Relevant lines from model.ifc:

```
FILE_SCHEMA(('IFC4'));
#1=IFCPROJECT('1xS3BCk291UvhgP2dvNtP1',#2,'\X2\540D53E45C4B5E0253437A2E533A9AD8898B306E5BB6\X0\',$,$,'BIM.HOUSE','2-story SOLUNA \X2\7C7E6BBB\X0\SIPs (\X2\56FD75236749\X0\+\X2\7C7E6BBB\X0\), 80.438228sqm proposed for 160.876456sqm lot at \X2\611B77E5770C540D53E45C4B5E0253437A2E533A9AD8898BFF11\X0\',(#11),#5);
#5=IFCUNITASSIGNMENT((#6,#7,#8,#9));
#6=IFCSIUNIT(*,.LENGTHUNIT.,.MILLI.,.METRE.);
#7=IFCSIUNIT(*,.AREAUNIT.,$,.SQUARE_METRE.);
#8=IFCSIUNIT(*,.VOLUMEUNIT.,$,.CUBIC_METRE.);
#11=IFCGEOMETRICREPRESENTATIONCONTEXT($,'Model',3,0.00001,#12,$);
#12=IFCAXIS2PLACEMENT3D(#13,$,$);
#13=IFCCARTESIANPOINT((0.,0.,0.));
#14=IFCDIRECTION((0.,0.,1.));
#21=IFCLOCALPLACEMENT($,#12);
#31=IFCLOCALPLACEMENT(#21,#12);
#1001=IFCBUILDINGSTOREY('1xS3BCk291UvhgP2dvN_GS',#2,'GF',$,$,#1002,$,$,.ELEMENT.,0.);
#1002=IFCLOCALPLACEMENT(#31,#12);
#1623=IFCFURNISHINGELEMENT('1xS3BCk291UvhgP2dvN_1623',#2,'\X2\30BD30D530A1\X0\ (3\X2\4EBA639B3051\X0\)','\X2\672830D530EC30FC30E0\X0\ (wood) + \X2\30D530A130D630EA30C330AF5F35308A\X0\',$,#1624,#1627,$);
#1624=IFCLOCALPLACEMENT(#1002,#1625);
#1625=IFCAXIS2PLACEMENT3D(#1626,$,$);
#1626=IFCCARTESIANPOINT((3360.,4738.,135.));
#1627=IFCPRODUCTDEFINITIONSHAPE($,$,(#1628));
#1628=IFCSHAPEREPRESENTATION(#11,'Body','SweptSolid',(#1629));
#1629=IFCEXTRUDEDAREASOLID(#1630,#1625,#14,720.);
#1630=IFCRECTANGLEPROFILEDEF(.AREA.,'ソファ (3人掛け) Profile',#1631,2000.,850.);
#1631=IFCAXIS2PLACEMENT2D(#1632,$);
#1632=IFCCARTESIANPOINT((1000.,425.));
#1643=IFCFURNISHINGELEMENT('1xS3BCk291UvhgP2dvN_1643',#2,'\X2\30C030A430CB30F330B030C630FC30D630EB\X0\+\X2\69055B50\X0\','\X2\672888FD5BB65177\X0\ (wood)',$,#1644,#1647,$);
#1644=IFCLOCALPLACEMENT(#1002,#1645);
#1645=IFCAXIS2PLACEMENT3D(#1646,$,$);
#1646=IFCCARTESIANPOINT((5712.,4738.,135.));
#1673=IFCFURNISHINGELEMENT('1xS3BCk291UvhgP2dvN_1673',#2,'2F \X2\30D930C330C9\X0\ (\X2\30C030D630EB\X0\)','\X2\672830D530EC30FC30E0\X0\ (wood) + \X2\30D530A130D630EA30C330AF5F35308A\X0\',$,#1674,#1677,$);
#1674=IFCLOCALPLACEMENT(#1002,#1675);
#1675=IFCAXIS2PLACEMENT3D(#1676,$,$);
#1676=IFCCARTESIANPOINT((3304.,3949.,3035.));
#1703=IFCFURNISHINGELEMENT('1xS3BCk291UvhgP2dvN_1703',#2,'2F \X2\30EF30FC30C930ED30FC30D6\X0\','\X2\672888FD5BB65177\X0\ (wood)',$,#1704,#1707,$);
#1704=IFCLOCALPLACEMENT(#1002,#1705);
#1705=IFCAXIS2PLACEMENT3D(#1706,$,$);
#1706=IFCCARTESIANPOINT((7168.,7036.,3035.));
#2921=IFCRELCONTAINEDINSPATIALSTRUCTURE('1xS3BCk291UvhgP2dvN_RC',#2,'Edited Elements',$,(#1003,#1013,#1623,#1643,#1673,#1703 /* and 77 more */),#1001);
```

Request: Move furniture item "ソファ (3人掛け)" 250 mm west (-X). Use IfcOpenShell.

```python
import ifcopenshell
import ifcopenshell.api.geometry
import ifcopenshell.util.placement
import ifcopenshell.util.unit

model = ifcopenshell.open("model.ifc")
unit_scale = ifcopenshell.util.unit.calculate_unit_scale(model)

item = model.by_guid("1xS3BCk291UvhgP2dvN_1623")
matrix = ifcopenshell.util.placement.get_local_placement(item.ObjectPlacement)
matrix[0, 3] -= 0.25 / unit_scale
ifcopenshell.api.geometry.edit_object_placement(model, product=item, matrix=matrix, is_si=False)

print(ifcopenshell.util.placement.get_local_placement(item.ObjectPlacement).round(3) + 0.0)

model.write("model_v2.ifc")
```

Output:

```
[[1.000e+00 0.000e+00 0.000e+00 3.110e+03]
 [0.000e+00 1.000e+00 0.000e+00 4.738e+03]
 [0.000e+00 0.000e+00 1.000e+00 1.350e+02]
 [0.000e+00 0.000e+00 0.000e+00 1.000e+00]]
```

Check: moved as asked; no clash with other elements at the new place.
